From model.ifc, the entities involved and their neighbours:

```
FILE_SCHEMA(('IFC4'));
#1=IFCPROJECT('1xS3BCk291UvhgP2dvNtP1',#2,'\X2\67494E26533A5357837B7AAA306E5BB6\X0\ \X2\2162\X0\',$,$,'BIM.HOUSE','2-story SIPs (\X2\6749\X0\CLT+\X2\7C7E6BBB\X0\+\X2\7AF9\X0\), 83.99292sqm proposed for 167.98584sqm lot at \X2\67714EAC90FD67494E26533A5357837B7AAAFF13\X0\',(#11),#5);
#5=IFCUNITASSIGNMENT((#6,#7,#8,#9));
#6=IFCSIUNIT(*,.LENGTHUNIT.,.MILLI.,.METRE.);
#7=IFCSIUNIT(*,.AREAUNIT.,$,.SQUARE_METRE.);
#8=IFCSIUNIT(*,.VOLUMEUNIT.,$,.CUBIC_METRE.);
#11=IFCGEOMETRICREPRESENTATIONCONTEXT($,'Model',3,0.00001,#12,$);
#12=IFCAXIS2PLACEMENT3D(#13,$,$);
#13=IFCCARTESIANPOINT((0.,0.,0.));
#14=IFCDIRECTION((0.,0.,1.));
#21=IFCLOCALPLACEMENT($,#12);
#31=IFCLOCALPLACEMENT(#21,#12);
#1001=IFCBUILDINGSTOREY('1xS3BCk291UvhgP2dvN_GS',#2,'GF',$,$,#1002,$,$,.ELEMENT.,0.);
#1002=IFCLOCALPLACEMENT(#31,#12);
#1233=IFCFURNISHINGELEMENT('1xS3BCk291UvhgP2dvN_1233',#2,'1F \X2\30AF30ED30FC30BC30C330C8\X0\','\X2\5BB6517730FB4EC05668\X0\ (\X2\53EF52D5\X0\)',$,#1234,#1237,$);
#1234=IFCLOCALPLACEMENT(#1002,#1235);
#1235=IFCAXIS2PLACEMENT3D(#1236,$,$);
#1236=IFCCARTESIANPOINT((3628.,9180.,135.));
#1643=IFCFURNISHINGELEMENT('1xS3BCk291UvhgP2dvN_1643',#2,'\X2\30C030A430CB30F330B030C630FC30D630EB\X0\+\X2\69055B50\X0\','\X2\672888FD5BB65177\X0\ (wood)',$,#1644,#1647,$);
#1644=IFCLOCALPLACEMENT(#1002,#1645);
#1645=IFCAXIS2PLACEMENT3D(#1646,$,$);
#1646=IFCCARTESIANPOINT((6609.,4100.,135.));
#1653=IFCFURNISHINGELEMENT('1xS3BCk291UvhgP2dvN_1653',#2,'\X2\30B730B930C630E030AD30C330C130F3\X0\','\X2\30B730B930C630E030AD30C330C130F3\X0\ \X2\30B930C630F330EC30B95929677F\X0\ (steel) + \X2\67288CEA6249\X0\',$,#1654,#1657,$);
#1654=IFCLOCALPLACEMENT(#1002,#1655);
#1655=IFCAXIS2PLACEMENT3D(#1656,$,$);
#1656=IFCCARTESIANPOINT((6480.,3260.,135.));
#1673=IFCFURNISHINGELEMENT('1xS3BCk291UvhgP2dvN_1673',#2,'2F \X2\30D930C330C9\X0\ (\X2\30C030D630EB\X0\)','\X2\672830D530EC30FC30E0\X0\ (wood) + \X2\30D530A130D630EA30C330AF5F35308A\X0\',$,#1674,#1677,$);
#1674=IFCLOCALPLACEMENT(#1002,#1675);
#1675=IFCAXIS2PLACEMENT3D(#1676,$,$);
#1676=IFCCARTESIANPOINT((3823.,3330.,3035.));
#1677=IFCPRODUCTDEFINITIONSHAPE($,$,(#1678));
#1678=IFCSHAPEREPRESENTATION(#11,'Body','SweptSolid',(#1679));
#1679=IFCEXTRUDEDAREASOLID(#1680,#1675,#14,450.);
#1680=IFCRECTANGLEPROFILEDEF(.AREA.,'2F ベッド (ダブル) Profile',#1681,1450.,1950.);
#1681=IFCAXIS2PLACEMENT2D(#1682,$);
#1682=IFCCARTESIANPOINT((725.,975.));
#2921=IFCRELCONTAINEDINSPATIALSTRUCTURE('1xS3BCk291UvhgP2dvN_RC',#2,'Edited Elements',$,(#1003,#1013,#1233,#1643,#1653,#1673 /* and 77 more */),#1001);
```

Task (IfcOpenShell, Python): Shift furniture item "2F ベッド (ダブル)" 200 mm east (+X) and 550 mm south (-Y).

```python
import ifcopenshell
import ifcopenshell.api.geometry
import ifcopenshell.util.placement
import ifcopenshell.util.unit

model = ifcopenshell.open("model.ifc")
unit_scale = ifcopenshell.util.unit.calculate_unit_scale(model)

item = model.by_guid("1xS3BCk291UvhgP2dvN_1673")
matrix = ifcopenshell.util.placement.get_local_placement(item.ObjectPlacement)
matrix[0, 3] += 0.2 / unit_scale
matrix[1, 3] -= 0.55 / unit_scale
ifcopenshell.api.geometry.edit_object_placement(model, product=item, matrix=matrix, is_si=False)

print(ifcopenshell.util.placement.get_local_placement(item.ObjectPlacement).round(3) + 0.0)

model.write("model-out.ifc")
```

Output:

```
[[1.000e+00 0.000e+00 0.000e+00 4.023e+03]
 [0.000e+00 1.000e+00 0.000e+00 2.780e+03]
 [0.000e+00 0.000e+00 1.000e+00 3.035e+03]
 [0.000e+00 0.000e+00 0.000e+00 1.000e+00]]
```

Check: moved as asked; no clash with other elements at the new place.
